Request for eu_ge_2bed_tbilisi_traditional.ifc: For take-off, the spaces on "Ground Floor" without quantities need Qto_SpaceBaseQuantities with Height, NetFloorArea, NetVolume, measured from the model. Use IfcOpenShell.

First a look at what the model holds.

```python
import ifcopenshell
import ifcopenshell.util.element
import ifcopenshell.util.unit

model = ifcopenshell.open("eu_ge_2bed_tbilisi_traditional.ifc")
print(model.schema)
for unit_type in ("LENGTHUNIT", "AREAUNIT", "VOLUMEUNIT"):
    print(unit_type, ifcopenshell.util.unit.calculate_unit_scale(model, unit_type))
storey = next(s for s in model.by_type("IfcBuildingStorey") if s.Name == "Ground Floor")
spaces = [e for e in ifcopenshell.util.element.get_decomposition(storey) if e.is_a("IfcSpace")]
for e in sorted(spaces, key=lambda e: e.id()):
    print(e.id(), e.is_a(), e.Name, list(ifcopenshell.util.element.get_psets(e, qtos_only=True)), sep=" | ")
```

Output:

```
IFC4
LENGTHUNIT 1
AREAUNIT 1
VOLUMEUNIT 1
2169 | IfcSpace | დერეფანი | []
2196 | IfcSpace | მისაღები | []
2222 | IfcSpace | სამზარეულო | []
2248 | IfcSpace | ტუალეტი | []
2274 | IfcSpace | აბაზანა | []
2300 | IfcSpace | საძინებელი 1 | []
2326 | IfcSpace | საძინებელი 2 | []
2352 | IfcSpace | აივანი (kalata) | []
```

```python
import ifcopenshell
import ifcopenshell.api.pset
import ifcopenshell.geom
import ifcopenshell.util.element
import ifcopenshell.util.shape
import ifcopenshell.util.unit

model = ifcopenshell.open("eu_ge_2bed_tbilisi_traditional.ifc")
unit_scale = ifcopenshell.util.unit.calculate_unit_scale(model)
area_scale = ifcopenshell.util.unit.calculate_unit_scale(model, "AREAUNIT")
volume_scale = ifcopenshell.util.unit.calculate_unit_scale(model, "VOLUMEUNIT")
settings = ifcopenshell.geom.settings()

storey = next(s for s in model.by_type("IfcBuildingStorey") if s.Name == "Ground Floor")
spaces = [e for e in ifcopenshell.util.element.get_decomposition(storey) if e.is_a("IfcSpace")]

for e in sorted(spaces, key=lambda e: e.id()):
    if ifcopenshell.util.element.get_psets(e, qtos_only=True, should_inherit=False):
        continue
    # Geometry comes back in metres, in the element's own axes.
    shape = ifcopenshell.geom.create_shape(settings, e)
    values = {
        "Height": ifcopenshell.util.shape.get_z(shape.geometry) / unit_scale,
        "NetFloorArea": ifcopenshell.util.shape.get_footprint_area(shape.geometry) / area_scale,
        "NetVolume": ifcopenshell.util.shape.get_volume(shape.geometry) / volume_scale,
    }
    qto = ifcopenshell.api.pset.add_qto(model, product=e, name="Qto_SpaceBaseQuantities")
    ifcopenshell.api.pset.edit_qto(model, qto=qto, properties=values)
    print(e.id(), {k: round(v, 3) for k, v in values.items()})

model.write("eu_ge_2bed_tbilisi_traditional_updated.ifc")
```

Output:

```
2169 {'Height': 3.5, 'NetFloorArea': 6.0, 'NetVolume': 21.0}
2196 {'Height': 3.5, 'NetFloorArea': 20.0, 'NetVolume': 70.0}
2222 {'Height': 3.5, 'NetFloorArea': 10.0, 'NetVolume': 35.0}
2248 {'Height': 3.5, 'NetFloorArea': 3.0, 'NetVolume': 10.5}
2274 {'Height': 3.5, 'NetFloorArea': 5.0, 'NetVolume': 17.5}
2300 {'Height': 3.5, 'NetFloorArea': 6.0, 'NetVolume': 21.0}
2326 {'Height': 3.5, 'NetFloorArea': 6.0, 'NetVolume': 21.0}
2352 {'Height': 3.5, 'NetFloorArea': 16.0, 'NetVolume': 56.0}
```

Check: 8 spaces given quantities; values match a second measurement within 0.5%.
